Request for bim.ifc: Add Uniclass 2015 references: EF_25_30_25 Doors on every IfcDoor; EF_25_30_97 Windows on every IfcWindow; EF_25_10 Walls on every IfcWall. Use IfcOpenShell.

First a look at what the model holds.

```python
import ifcopenshell

model = ifcopenshell.open("bim.ifc")
print(model.schema)
print("classifications:", [c.Name for c in model.by_type("IfcClassification")])
for ifc_class in ("IfcDoor", "IfcRoof", "IfcStair", "IfcWall", "IfcWindow"):
    print(ifc_class, len(model.by_type(ifc_class)))
```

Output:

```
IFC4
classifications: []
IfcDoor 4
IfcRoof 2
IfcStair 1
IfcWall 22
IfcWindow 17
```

```python
import ifcopenshell
import ifcopenshell.api.classification

model = ifcopenshell.open("bim.ifc")

system = ifcopenshell.api.classification.add_classification(model, classification="Uniclass 2015")

codes = {
    "IfcDoor": ("EF_25_30_25", "Doors"),
    "IfcWindow": ("EF_25_30_97", "Windows"),
    "IfcWall": ("EF_25_10", "Walls"),
}
for ifc_class, (code, name) in codes.items():
    products = model.by_type(ifc_class)
    ifcopenshell.api.classification.add_reference(
        model, products=products, classification=system, identification=code, name=name
    )
    print(code, len(products))

model.write("bim_v2.ifc")
```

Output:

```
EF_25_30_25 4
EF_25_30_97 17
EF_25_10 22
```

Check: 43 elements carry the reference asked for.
